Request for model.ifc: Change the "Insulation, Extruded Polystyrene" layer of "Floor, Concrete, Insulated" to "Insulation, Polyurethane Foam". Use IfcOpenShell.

First a look at what the model holds.

```python
import ifcopenshell
import ifcopenshell.util.element

model = ifcopenshell.open("model.ifc")
print(model.schema)
for layer_set in model.by_type("IfcMaterialLayerSet"):
    if layer_set.LayerSetName == "Floor, Concrete, Insulated":
        for layer in layer_set.MaterialLayers:
            print(layer.id(), layer.Material and layer.Material.Name, layer.LayerThickness, sep=" | ")
        print(len(ifcopenshell.util.element.get_elements_by_material(model, layer_set)), "elements and types use it")
print(sorted(m.Name for m in model.by_type("IfcMaterial") if m.Name)[:60])
```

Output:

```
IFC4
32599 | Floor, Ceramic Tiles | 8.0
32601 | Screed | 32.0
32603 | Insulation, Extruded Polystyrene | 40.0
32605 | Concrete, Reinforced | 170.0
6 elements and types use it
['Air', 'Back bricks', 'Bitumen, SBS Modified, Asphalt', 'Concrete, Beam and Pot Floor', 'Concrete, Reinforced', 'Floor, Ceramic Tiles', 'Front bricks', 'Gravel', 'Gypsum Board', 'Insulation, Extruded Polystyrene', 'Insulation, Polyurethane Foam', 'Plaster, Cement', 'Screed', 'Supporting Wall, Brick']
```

```python
import ifcopenshell
import ifcopenshell.api.material

model = ifcopenshell.open("model.ifc")

layer_set = next(s for s in model.by_type("IfcMaterialLayerSet") if s.LayerSetName == "Floor, Concrete, Insulated")
layer = next(l for l in layer_set.MaterialLayers if l.Material and l.Material.Name == "Insulation, Extruded Polystyrene")
material = next(m for m in model.by_type("IfcMaterial") if m.Name == "Insulation, Polyurethane Foam")

# Point this one layer at the other material; renaming the old one would change it everywhere.
ifcopenshell.api.material.edit_layer(model, layer=layer, attributes={}, material=material)

print([l.Material.Name if l.Material else None for l in layer_set.MaterialLayers])

model.write("model_edited.ifc")
```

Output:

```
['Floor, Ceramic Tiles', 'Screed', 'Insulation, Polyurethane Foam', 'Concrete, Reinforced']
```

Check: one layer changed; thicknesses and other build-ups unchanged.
